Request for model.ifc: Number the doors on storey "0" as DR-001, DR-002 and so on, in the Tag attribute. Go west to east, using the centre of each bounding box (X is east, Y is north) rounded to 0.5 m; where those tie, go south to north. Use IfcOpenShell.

First a look at what the model holds.

```python
import ifcopenshell
import ifcopenshell.util.element
import ifcopenshell.util.placement

model = ifcopenshell.open("model.ifc")
print(model.schema)
storey = next(s for s in model.by_type("IfcBuildingStorey") if s.Name == "0")
doors = [e for e in ifcopenshell.util.element.get_decomposition(storey) if e.is_a("IfcDoor")]
for e in sorted(doors, key=lambda e: e.id()):
    origin = ifcopenshell.util.placement.get_local_placement(e.ObjectPlacement)[:3, 3]
    print(e.id(), e.Tag, e.Name, origin.round(2) + 0.0, sep=" | ")
```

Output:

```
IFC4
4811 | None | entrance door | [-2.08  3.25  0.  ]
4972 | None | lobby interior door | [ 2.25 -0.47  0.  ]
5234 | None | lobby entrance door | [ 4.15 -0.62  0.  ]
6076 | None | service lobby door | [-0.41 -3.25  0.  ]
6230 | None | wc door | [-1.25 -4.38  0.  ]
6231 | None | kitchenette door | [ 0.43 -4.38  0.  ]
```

```python
import ifcopenshell
import ifcopenshell.geom
import ifcopenshell.util.element
import ifcopenshell.util.shape

model = ifcopenshell.open("model.ifc")
settings = ifcopenshell.geom.settings()
settings.set("use-world-coords", True)


def centre(element):
    shape = ifcopenshell.geom.create_shape(settings, element)
    return ifcopenshell.util.shape.get_bbox_centroid(shape.geometry)


storey = next(s for s in model.by_type("IfcBuildingStorey") if s.Name == "0")
doors = [e for e in ifcopenshell.util.element.get_decomposition(storey) if e.is_a("IfcDoor")]

# Insertion points can sit at a corner or the storey origin, so sort by the geometry (in metres).
centres = {e: centre(e) for e in doors}
doors.sort(key=lambda e: (round(centres[e][0] / 0.5), centres[e][1]))

for i, e in enumerate(doors, start=1):
    number = f"DR-0{i:02d}"
    e.Tag = number
    print(e.id(), number)

model.write("model-out.ifc")
```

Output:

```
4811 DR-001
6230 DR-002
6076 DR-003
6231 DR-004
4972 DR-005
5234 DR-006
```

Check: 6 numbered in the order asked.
